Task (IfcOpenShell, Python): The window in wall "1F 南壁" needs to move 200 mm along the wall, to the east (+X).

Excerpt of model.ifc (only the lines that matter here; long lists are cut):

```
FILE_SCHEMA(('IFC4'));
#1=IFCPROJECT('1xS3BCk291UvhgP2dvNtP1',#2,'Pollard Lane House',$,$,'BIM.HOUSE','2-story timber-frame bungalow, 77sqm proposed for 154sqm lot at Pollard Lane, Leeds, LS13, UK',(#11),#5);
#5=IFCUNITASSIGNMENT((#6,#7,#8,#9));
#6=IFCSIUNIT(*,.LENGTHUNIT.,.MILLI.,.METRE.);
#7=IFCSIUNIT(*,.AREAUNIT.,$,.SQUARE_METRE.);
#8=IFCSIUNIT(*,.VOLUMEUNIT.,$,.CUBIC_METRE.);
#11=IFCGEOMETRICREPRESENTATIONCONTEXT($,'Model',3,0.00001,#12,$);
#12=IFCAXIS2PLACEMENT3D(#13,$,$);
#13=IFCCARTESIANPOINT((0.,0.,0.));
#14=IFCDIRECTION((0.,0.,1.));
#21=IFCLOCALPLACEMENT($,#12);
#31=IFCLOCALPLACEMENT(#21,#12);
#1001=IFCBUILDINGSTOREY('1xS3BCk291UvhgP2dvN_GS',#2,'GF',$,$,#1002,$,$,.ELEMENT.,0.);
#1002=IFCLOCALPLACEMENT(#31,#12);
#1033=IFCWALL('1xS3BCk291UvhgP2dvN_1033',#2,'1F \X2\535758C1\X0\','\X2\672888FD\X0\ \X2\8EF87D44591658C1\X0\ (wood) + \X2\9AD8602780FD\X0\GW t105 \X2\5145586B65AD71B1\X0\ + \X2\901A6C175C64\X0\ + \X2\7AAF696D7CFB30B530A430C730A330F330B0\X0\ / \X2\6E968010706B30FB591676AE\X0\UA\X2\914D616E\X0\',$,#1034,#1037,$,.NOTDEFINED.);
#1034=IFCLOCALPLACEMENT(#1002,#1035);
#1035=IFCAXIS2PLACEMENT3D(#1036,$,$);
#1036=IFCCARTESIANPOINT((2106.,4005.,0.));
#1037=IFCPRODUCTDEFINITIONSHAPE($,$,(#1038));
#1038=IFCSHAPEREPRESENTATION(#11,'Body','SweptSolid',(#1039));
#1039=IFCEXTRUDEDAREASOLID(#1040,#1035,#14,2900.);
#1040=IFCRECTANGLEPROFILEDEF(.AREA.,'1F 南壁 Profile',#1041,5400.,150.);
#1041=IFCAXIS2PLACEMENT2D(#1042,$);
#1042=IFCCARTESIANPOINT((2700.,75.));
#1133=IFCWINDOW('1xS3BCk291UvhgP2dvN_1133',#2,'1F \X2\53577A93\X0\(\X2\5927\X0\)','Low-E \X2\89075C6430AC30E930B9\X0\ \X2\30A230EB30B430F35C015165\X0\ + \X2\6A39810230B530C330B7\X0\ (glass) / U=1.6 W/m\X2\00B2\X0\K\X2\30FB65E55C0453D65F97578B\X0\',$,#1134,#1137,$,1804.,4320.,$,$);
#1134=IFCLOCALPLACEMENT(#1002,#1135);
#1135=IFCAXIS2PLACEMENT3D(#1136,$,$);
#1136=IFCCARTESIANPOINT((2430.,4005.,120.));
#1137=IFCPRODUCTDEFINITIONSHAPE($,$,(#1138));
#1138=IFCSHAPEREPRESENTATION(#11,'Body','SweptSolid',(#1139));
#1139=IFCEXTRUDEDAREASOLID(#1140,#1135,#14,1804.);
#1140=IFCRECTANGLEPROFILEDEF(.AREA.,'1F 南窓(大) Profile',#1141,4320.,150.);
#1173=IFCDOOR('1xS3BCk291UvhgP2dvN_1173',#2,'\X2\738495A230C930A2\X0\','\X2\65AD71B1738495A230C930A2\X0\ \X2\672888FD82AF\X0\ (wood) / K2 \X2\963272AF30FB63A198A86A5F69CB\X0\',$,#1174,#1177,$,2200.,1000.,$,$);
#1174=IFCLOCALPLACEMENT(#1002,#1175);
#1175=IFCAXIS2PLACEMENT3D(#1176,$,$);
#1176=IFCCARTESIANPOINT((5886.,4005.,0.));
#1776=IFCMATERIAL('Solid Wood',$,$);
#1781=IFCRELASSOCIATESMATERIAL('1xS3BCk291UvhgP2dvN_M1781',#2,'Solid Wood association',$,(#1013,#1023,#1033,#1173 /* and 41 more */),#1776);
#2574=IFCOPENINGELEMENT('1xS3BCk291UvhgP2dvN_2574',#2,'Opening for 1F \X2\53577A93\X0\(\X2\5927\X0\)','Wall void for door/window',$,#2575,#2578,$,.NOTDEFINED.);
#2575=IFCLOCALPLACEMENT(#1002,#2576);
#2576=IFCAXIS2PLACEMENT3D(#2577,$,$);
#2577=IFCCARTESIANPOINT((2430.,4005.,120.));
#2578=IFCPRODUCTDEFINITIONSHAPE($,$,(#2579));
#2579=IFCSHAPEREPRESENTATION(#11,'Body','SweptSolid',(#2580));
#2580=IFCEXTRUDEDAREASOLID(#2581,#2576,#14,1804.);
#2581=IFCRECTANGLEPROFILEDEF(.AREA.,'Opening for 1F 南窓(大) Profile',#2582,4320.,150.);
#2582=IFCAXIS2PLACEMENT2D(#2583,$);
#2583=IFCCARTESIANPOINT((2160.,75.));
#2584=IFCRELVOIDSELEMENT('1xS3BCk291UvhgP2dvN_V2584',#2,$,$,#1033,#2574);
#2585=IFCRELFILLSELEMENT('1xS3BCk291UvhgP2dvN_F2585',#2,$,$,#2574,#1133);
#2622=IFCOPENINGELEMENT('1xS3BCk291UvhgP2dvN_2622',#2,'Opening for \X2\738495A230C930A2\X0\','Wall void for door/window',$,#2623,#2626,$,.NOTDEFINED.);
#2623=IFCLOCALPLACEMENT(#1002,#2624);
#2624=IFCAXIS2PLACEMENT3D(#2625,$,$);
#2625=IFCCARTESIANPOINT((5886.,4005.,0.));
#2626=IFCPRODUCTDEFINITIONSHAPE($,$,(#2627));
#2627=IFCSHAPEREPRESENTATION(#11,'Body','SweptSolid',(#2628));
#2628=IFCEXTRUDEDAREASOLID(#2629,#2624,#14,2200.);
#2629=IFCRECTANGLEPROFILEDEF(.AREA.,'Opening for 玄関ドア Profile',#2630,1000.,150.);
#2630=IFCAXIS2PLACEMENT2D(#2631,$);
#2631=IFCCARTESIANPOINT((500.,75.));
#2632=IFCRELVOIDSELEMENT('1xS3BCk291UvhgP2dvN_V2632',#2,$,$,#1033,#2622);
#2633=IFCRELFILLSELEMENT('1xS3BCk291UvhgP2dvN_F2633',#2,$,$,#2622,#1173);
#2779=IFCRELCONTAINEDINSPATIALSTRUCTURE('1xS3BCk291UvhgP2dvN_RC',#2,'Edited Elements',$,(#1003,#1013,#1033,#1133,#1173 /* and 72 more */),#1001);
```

```python
import ifcopenshell
import ifcopenshell.api.geometry
import ifcopenshell.util.placement
import ifcopenshell.util.unit

model = ifcopenshell.open("model.ifc")
unit_scale = ifcopenshell.util.unit.calculate_unit_scale(model)

window = model.by_guid("1xS3BCk291UvhgP2dvN_1133")
opening = window.FillsVoids[0].RelatingOpeningElement
wall = opening.VoidsElements[0].RelatingBuildingElement

wall_matrix = ifcopenshell.util.placement.get_local_placement(wall.ObjectPlacement)
shift = wall_matrix[:3, 0] * 0.2 / unit_scale
before = ifcopenshell.util.placement.get_local_placement(window.ObjectPlacement)[:3, 3].copy()

# The window is not placed relative to its opening, so move both.
for product in (opening, window):
    matrix = ifcopenshell.util.placement.get_local_placement(product.ObjectPlacement)
    matrix[:3, 3] += shift
    ifcopenshell.api.geometry.edit_object_placement(model, product=product, matrix=matrix, is_si=False)

after = ifcopenshell.util.placement.get_local_placement(window.ObjectPlacement)[:3, 3]
print("window moved by", (after - before).round(3) + 0.0)

model.write("model_v2.ifc")
```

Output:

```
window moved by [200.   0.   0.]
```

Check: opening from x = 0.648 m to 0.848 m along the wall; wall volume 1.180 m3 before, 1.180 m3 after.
